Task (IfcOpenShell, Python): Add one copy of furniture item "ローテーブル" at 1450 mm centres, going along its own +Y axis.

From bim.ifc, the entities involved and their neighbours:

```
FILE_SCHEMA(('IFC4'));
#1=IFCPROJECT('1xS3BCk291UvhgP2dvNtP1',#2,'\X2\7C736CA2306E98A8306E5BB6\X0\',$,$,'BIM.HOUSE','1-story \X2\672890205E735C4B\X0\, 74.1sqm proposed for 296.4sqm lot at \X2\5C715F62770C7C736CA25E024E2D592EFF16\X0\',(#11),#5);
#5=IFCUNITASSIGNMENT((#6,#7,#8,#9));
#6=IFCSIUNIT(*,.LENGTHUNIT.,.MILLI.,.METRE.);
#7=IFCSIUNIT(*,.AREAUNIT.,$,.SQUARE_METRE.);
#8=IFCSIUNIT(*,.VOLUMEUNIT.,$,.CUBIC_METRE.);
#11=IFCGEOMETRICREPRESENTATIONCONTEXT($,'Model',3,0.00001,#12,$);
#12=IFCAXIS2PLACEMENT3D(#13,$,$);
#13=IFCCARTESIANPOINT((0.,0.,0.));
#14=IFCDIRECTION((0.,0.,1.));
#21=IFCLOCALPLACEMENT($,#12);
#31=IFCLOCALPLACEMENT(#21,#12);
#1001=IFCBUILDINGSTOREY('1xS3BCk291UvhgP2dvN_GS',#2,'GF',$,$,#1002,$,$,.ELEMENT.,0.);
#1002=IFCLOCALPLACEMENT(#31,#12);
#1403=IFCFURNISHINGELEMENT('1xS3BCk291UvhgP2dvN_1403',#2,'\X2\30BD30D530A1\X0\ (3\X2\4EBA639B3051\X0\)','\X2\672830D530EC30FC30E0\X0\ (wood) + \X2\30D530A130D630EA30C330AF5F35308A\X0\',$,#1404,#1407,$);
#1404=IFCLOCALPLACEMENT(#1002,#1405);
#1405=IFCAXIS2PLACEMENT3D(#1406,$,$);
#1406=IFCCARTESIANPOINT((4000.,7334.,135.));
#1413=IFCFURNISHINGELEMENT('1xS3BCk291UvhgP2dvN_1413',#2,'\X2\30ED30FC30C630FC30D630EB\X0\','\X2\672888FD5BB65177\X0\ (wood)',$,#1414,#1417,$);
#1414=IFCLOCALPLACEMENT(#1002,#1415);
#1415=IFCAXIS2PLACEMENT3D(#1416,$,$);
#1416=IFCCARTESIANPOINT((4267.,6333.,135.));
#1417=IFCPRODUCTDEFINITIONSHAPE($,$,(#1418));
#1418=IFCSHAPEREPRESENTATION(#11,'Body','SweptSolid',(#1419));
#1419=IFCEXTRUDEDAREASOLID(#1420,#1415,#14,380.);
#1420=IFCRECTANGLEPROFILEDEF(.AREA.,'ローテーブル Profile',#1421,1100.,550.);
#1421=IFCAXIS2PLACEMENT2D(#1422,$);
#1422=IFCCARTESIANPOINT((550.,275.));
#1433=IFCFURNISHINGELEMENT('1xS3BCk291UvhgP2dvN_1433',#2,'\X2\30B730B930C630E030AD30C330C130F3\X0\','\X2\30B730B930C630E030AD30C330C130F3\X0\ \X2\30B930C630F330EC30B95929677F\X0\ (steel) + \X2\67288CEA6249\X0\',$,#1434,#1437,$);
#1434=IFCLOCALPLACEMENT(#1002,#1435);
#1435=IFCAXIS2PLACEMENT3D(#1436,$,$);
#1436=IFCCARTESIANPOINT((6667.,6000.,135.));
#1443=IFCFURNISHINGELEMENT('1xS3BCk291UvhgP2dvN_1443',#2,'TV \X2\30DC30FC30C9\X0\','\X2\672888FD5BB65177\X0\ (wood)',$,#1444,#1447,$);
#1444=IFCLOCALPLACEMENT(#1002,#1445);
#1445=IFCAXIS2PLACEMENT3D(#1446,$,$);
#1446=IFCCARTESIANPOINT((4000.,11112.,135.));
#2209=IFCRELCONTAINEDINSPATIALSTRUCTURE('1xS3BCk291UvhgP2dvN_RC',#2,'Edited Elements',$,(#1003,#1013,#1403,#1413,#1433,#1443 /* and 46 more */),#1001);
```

```python
import ifcopenshell
import ifcopenshell.api.geometry
import ifcopenshell.api.root
import ifcopenshell.util.element
import ifcopenshell.util.placement
import ifcopenshell.util.unit

model = ifcopenshell.open("bim.ifc")
unit_scale = ifcopenshell.util.unit.calculate_unit_scale(model)


def reuse_history(source, copy):
    """copy_class also copies each property set's owner history, people and application; keep the originals."""
    for rel in copy.IsDefinedBy:
        if rel.is_a("IfcRelDefinesByProperties") and (history := rel.RelatingPropertyDefinition.OwnerHistory):
            rel.RelatingPropertyDefinition.OwnerHistory = source.OwnerHistory
            ifcopenshell.util.element.remove_deep2(model, history)


source = model.by_guid("1xS3BCk291UvhgP2dvN_1413")
base = ifcopenshell.util.placement.get_local_placement(source.ObjectPlacement)
step = base[:3, 1] * 1.45 / unit_scale

for i in range(1, 2):
    copy = ifcopenshell.api.root.copy_class(model, product=source)
    copy.Representation = ifcopenshell.util.element.copy_deep(
        model, source.Representation, exclude=["IfcGeometricRepresentationContext", "IfcRepresentationMap"]
    )
    reuse_history(source, copy)
    matrix = base.copy()
    matrix[:3, 3] += i * step
    print("added at", matrix[:3, 3].round(3) + 0.0)
    ifcopenshell.api.geometry.edit_object_placement(model, product=copy, matrix=matrix, is_si=False)

model.write("bim_v2.ifc")
```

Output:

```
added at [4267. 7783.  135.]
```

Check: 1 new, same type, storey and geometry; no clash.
